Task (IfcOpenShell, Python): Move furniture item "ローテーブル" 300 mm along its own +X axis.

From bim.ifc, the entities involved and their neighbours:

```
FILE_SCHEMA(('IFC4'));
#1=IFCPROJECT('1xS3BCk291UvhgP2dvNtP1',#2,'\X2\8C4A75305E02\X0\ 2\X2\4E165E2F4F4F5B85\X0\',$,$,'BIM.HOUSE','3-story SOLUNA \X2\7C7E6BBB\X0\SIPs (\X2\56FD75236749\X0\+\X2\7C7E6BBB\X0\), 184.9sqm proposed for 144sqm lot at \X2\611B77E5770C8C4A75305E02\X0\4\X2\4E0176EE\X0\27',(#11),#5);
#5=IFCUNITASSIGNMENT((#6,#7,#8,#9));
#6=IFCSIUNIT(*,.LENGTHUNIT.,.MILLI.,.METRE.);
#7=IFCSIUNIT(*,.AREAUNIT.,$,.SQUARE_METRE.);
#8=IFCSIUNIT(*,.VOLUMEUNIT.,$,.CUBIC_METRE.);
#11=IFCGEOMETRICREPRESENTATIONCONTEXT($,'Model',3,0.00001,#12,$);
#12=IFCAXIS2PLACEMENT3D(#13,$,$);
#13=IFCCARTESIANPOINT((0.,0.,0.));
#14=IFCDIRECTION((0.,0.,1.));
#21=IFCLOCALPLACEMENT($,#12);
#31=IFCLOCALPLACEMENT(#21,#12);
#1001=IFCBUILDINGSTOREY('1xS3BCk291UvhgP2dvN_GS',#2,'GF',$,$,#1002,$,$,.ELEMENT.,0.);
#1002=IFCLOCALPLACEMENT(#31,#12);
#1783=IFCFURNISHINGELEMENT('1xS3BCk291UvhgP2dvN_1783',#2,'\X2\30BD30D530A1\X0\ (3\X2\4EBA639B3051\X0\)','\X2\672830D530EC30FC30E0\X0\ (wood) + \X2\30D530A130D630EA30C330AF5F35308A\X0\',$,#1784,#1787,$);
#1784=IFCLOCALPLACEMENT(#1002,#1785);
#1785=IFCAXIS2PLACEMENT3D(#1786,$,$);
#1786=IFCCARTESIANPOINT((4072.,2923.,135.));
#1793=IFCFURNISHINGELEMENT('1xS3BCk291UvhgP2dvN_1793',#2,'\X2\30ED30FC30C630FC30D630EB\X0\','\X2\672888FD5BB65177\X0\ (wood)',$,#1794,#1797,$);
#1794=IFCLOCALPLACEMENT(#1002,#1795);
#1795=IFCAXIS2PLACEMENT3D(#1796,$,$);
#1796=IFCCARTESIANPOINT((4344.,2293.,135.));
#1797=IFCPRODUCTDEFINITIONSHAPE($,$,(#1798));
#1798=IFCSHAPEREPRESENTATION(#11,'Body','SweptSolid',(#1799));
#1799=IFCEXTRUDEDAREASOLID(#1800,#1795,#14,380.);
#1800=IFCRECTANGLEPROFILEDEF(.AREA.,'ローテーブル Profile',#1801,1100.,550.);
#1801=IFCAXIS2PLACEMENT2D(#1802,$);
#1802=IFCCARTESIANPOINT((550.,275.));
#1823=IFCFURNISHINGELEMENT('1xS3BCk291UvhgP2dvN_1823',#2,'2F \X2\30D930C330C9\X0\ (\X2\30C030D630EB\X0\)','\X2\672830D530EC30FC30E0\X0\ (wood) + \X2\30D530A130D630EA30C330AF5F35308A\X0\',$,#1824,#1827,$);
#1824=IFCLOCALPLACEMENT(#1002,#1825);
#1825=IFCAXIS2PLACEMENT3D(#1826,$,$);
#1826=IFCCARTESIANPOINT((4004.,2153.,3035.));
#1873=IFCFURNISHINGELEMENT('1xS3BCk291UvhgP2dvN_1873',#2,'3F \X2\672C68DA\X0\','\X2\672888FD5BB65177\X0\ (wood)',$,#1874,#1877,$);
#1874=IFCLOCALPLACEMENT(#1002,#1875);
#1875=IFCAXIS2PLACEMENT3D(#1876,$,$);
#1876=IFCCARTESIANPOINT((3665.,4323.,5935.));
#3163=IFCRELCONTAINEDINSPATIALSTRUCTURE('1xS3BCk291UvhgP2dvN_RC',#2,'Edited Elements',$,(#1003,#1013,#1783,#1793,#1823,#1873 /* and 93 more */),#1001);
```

```python
import ifcopenshell
import ifcopenshell.api.geometry
import ifcopenshell.util.placement
import ifcopenshell.util.unit

model = ifcopenshell.open("bim.ifc")
unit_scale = ifcopenshell.util.unit.calculate_unit_scale(model)

item = model.by_guid("1xS3BCk291UvhgP2dvN_1793")
matrix = ifcopenshell.util.placement.get_local_placement(item.ObjectPlacement)
matrix[:3, 3] += matrix[:3, 0] * 0.3 / unit_scale
ifcopenshell.api.geometry.edit_object_placement(model, product=item, matrix=matrix, is_si=False)

print(ifcopenshell.util.placement.get_local_placement(item.ObjectPlacement).round(3) + 0.0)

model.write("bim_updated.ifc")
```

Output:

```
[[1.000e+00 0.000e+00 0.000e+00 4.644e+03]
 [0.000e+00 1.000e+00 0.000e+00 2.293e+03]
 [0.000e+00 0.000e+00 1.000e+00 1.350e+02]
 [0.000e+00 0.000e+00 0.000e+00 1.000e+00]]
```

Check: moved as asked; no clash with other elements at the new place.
